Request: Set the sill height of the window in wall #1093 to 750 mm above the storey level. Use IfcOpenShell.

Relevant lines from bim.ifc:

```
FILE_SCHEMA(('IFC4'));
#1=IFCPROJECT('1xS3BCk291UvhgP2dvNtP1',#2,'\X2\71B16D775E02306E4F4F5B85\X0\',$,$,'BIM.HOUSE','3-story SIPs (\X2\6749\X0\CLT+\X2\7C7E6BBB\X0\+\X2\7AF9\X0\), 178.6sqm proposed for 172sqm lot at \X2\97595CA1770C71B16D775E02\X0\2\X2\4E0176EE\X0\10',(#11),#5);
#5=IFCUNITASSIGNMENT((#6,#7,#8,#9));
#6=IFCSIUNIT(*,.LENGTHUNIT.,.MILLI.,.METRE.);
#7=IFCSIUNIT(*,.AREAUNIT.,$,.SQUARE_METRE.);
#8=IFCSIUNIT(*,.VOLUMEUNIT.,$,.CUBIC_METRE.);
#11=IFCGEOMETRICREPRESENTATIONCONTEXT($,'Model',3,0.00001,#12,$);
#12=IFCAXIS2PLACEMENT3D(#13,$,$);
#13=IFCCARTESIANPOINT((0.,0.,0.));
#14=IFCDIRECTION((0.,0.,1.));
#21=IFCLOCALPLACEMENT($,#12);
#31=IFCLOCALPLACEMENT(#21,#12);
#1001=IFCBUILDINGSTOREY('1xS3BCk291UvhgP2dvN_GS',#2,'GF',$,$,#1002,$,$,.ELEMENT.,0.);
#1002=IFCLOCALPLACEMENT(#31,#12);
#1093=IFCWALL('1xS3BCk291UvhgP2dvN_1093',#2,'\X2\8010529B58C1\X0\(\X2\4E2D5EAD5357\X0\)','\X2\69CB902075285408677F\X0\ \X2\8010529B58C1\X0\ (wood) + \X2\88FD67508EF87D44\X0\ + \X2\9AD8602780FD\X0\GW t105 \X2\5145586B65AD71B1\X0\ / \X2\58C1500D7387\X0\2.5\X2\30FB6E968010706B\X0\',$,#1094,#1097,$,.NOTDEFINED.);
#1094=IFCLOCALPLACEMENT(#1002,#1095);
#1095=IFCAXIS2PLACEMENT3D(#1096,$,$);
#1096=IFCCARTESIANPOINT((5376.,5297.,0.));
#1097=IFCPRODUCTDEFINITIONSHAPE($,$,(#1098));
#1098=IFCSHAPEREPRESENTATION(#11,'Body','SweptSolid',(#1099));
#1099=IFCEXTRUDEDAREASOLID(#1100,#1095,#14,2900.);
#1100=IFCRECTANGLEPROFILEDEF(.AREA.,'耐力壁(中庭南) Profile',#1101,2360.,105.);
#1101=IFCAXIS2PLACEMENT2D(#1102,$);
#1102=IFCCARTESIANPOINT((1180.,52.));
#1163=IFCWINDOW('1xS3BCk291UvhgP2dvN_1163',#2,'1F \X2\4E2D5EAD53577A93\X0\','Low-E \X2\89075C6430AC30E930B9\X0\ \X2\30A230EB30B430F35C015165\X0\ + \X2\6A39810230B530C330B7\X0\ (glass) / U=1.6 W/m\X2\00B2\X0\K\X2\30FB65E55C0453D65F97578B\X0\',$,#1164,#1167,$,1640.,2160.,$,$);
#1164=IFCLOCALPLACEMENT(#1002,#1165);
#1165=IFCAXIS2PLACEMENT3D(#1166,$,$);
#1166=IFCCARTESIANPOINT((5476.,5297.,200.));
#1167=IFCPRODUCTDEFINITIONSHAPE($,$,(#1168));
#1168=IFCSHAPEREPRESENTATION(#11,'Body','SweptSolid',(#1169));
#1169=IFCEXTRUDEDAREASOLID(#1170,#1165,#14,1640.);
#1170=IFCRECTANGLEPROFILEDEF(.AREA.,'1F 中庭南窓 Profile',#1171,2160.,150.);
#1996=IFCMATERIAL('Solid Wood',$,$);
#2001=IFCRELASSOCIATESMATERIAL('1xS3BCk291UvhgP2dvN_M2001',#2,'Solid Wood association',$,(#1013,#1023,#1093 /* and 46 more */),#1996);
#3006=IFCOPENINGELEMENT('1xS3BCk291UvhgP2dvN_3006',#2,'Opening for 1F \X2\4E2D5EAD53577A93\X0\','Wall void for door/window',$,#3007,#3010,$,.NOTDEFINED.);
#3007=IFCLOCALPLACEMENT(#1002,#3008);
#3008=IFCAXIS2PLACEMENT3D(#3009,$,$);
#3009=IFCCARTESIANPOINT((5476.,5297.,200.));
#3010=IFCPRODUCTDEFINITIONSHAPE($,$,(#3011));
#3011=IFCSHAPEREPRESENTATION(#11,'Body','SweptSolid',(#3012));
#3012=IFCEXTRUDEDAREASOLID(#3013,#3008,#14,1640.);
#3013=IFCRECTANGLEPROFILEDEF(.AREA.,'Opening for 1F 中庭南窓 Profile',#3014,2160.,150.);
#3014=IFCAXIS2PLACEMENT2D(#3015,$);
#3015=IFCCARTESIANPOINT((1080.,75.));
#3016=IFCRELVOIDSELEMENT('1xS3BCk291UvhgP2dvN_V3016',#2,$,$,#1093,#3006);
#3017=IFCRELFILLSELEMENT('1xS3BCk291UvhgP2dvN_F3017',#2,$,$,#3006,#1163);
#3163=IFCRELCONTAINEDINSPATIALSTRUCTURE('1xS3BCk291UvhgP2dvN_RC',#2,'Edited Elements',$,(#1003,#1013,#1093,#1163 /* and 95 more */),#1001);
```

```python
import numpy as np
import ifcopenshell
import ifcopenshell.api.geometry
import ifcopenshell.geom
import ifcopenshell.util.element
import ifcopenshell.util.placement
import ifcopenshell.util.shape
import ifcopenshell.util.unit

model = ifcopenshell.open("bim.ifc")
unit_scale = ifcopenshell.util.unit.calculate_unit_scale(model)

window = model.by_id(1163)
opening = window.FillsVoids[0].RelatingOpeningElement
storey = ifcopenshell.util.element.get_container(window, ifc_class="IfcBuildingStorey")
level = ifcopenshell.util.placement.get_local_placement(storey.ObjectPlacement)[2, 3]

# The opening's origin need not be at the sill, so measure its lowest point.
shape = ifcopenshell.geom.create_shape(ifcopenshell.geom.settings(), opening)
bottom = ifcopenshell.util.shape.get_shape_bottom_elevation(shape, shape.geometry) / unit_scale
dz = level + 0.75 / unit_scale - bottom

shift = np.array([0.0, 0.0, dz])
# The window is not placed relative to its opening, so move both.
for product in (opening, window):
    matrix = ifcopenshell.util.placement.get_local_placement(product.ObjectPlacement)
    matrix[:3, 3] += shift
    ifcopenshell.api.geometry.edit_object_placement(model, product=product, matrix=matrix, is_si=False)

print(f"moved by {dz * unit_scale:+.3f} m")

model.write("bim_updated.ifc")
```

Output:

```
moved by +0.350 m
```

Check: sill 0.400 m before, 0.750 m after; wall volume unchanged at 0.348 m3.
